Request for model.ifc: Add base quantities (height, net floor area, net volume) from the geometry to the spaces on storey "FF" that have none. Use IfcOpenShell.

First a look at what the model holds.

```python
import ifcopenshell
import ifcopenshell.util.element
import ifcopenshell.util.unit

model = ifcopenshell.open("model.ifc")
print(model.schema)
for unit_type in ("LENGTHUNIT", "AREAUNIT", "VOLUMEUNIT"):
    print(unit_type, ifcopenshell.util.unit.calculate_unit_scale(model, unit_type))
storey = next(s for s in model.by_type("IfcBuildingStorey") if s.Name == "FF")
spaces = [e for e in ifcopenshell.util.element.get_decomposition(storey) if e.is_a("IfcSpace")]
for e in sorted(spaces, key=lambda e: e.id()):
    print(e.id(), e.is_a(), e.Name, list(ifcopenshell.util.element.get_psets(e, qtos_only=True)), sep=" | ")
```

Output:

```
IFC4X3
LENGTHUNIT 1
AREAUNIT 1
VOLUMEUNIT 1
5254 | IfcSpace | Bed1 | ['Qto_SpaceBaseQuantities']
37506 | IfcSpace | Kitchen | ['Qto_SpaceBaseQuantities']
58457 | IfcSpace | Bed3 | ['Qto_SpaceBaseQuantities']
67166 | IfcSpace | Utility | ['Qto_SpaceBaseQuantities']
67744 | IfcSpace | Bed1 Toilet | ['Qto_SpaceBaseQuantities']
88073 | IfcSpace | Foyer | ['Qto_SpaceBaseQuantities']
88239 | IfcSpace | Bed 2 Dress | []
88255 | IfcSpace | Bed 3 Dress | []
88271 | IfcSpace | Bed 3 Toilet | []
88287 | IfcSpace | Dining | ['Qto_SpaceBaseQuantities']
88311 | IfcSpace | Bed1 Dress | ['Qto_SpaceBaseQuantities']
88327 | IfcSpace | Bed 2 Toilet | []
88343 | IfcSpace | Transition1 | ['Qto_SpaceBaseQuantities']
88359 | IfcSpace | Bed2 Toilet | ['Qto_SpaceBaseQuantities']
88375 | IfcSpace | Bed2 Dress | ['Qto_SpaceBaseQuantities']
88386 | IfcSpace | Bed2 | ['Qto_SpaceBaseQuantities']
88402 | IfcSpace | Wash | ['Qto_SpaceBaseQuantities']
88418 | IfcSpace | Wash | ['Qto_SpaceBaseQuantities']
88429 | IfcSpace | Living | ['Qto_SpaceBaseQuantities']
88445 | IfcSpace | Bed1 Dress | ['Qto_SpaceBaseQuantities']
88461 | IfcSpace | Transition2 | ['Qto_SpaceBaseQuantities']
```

```python
import ifcopenshell
import ifcopenshell.api.pset
import ifcopenshell.geom
import ifcopenshell.util.element
import ifcopenshell.util.shape
import ifcopenshell.util.unit

model = ifcopenshell.open("model.ifc")
unit_scale = ifcopenshell.util.unit.calculate_unit_scale(model)
area_scale = ifcopenshell.util.unit.calculate_unit_scale(model, "AREAUNIT")
volume_scale = ifcopenshell.util.unit.calculate_unit_scale(model, "VOLUMEUNIT")
settings = ifcopenshell.geom.settings()

storey = next(s for s in model.by_type("IfcBuildingStorey") if s.Name == "FF")
spaces = [e for e in ifcopenshell.util.element.get_decomposition(storey) if e.is_a("IfcSpace")]

for e in sorted(spaces, key=lambda e: e.id()):
    if ifcopenshell.util.element.get_psets(e, qtos_only=True, should_inherit=False):
        continue
    # Geometry comes back in metres, in the element's own axes.
    shape = ifcopenshell.geom.create_shape(settings, e)
    values = {
        "Height": ifcopenshell.util.shape.get_z(shape.geometry) / unit_scale,
        "NetFloorArea": ifcopenshell.util.shape.get_footprint_area(shape.geometry) / area_scale,
        "NetVolume": ifcopenshell.util.shape.get_volume(shape.geometry) / volume_scale,
    }
    qto = ifcopenshell.api.pset.add_qto(model, product=e, name="Qto_SpaceBaseQuantities")
    ifcopenshell.api.pset.edit_qto(model, qto=qto, properties=values)
    print(e.id(), {k: round(v, 3) for k, v in values.items()})

model.write("model_rev.ifc")
```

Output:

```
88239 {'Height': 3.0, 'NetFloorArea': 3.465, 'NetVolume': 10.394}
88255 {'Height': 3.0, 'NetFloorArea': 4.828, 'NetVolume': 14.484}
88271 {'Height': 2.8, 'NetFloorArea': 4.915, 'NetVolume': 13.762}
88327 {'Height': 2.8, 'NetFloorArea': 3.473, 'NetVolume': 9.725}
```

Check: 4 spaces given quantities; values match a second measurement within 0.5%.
